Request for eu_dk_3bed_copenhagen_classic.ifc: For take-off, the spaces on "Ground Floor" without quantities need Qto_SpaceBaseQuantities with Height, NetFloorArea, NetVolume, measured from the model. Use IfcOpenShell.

First a look at what the model holds.

```python
import ifcopenshell
import ifcopenshell.util.element
import ifcopenshell.util.unit

model = ifcopenshell.open("eu_dk_3bed_copenhagen_classic.ifc")
print(model.schema)
for unit_type in ("LENGTHUNIT", "AREAUNIT", "VOLUMEUNIT"):
    print(unit_type, ifcopenshell.util.unit.calculate_unit_scale(model, unit_type))
storey = next(s for s in model.by_type("IfcBuildingStorey") if s.Name == "Ground Floor")
spaces = [e for e in ifcopenshell.util.element.get_decomposition(storey) if e.is_a("IfcSpace")]
for e in sorted(spaces, key=lambda e: e.id()):
    print(e.id(), e.is_a(), e.Name, list(ifcopenshell.util.element.get_psets(e, qtos_only=True)), sep=" | ")
```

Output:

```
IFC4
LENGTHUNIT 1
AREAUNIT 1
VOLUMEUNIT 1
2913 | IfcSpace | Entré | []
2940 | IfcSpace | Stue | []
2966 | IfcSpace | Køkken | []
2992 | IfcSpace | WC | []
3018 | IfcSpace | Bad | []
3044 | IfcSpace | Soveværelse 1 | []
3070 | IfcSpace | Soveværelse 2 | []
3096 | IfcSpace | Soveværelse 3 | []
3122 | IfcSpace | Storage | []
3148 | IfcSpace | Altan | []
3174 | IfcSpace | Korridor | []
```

```python
import ifcopenshell
import ifcopenshell.api.pset
import ifcopenshell.geom
import ifcopenshell.util.element
import ifcopenshell.util.shape
import ifcopenshell.util.unit

model = ifcopenshell.open("eu_dk_3bed_copenhagen_classic.ifc")
unit_scale = ifcopenshell.util.unit.calculate_unit_scale(model)
area_scale = ifcopenshell.util.unit.calculate_unit_scale(model, "AREAUNIT")
volume_scale = ifcopenshell.util.unit.calculate_unit_scale(model, "VOLUMEUNIT")
settings = ifcopenshell.geom.settings()

storey = next(s for s in model.by_type("IfcBuildingStorey") if s.Name == "Ground Floor")
spaces = [e for e in ifcopenshell.util.element.get_decomposition(storey) if e.is_a("IfcSpace")]

for e in sorted(spaces, key=lambda e: e.id()):
    if ifcopenshell.util.element.get_psets(e, qtos_only=True, should_inherit=False):
        continue
    # Geometry comes back in metres, in the element's own axes.
    shape = ifcopenshell.geom.create_shape(settings, e)
    values = {
        "Height": ifcopenshell.util.shape.get_z(shape.geometry) / unit_scale,
        "NetFloorArea": ifcopenshell.util.shape.get_footprint_area(shape.geometry) / area_scale,
        "NetVolume": ifcopenshell.util.shape.get_volume(shape.geometry) / volume_scale,
    }
    qto = ifcopenshell.api.pset.add_qto(model, product=e, name="Qto_SpaceBaseQuantities")
    ifcopenshell.api.pset.edit_qto(model, qto=qto, properties=values)
    print(e.id(), {k: round(v, 3) for k, v in values.items()})

model.write("eu_dk_3bed_copenhagen_classic_updated.ifc")
```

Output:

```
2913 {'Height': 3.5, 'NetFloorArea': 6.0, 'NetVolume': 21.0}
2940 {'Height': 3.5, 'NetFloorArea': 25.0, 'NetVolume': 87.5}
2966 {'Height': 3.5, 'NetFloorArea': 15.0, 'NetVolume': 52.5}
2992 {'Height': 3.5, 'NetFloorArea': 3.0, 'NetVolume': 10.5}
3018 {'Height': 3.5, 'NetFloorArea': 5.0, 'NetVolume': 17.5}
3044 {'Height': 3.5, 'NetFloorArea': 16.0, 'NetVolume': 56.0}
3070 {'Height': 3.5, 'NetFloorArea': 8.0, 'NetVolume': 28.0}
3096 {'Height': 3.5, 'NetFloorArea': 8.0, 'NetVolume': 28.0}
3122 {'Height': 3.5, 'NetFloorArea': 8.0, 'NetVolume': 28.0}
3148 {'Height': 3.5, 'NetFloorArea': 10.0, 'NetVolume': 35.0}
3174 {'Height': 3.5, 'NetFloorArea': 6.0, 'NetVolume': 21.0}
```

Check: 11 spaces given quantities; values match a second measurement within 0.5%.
